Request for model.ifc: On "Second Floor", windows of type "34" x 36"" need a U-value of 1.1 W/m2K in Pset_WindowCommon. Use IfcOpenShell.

First a look at what the model holds.

```python
import ifcopenshell
import ifcopenshell.util.element

model = ifcopenshell.open("model.ifc")
print(model.schema)
storey = next(s for s in model.by_type("IfcBuildingStorey") if s.Name == "Second Floor")
windows = [e for e in ifcopenshell.util.element.get_decomposition(storey) if e.is_a("IfcWindow")]
seen = {}
for e in windows:
    element_type = ifcopenshell.util.element.get_type(e)
    key = (element_type.Name if element_type != e and element_type else None, ifcopenshell.util.element.get_pset(e, "Pset_WindowCommon", "ThermalTransmittance"))
    seen[key] = seen.get(key, 0) + 1
for (name, value), count in sorted(seen.items(), key=str):
    print(count, "x", name, "|", value)
```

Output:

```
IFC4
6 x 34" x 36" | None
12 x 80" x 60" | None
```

```python
import ifcopenshell
import ifcopenshell.api.pset
import ifcopenshell.util.element

model = ifcopenshell.open("model.ifc")

storey = next(s for s in model.by_type("IfcBuildingStorey") if s.Name == "Second Floor")
windows = [e for e in ifcopenshell.util.element.get_decomposition(storey) if e.is_a("IfcWindow")]

count = 0
for e in windows:
    element_type = ifcopenshell.util.element.get_type(e)
    if element_type in (None, e) or element_type.Name != '34" x 36"':
        continue
    # add_pset returns the element's existing set when there is one.
    pset = ifcopenshell.api.pset.add_pset(model, product=e, name="Pset_WindowCommon")
    ifcopenshell.api.pset.edit_pset(model, pset=pset, properties={"ThermalTransmittance": 1.1})
    count += 1

print(count, "windows updated")

model.write("model_v2.ifc")
```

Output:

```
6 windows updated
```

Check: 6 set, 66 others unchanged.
